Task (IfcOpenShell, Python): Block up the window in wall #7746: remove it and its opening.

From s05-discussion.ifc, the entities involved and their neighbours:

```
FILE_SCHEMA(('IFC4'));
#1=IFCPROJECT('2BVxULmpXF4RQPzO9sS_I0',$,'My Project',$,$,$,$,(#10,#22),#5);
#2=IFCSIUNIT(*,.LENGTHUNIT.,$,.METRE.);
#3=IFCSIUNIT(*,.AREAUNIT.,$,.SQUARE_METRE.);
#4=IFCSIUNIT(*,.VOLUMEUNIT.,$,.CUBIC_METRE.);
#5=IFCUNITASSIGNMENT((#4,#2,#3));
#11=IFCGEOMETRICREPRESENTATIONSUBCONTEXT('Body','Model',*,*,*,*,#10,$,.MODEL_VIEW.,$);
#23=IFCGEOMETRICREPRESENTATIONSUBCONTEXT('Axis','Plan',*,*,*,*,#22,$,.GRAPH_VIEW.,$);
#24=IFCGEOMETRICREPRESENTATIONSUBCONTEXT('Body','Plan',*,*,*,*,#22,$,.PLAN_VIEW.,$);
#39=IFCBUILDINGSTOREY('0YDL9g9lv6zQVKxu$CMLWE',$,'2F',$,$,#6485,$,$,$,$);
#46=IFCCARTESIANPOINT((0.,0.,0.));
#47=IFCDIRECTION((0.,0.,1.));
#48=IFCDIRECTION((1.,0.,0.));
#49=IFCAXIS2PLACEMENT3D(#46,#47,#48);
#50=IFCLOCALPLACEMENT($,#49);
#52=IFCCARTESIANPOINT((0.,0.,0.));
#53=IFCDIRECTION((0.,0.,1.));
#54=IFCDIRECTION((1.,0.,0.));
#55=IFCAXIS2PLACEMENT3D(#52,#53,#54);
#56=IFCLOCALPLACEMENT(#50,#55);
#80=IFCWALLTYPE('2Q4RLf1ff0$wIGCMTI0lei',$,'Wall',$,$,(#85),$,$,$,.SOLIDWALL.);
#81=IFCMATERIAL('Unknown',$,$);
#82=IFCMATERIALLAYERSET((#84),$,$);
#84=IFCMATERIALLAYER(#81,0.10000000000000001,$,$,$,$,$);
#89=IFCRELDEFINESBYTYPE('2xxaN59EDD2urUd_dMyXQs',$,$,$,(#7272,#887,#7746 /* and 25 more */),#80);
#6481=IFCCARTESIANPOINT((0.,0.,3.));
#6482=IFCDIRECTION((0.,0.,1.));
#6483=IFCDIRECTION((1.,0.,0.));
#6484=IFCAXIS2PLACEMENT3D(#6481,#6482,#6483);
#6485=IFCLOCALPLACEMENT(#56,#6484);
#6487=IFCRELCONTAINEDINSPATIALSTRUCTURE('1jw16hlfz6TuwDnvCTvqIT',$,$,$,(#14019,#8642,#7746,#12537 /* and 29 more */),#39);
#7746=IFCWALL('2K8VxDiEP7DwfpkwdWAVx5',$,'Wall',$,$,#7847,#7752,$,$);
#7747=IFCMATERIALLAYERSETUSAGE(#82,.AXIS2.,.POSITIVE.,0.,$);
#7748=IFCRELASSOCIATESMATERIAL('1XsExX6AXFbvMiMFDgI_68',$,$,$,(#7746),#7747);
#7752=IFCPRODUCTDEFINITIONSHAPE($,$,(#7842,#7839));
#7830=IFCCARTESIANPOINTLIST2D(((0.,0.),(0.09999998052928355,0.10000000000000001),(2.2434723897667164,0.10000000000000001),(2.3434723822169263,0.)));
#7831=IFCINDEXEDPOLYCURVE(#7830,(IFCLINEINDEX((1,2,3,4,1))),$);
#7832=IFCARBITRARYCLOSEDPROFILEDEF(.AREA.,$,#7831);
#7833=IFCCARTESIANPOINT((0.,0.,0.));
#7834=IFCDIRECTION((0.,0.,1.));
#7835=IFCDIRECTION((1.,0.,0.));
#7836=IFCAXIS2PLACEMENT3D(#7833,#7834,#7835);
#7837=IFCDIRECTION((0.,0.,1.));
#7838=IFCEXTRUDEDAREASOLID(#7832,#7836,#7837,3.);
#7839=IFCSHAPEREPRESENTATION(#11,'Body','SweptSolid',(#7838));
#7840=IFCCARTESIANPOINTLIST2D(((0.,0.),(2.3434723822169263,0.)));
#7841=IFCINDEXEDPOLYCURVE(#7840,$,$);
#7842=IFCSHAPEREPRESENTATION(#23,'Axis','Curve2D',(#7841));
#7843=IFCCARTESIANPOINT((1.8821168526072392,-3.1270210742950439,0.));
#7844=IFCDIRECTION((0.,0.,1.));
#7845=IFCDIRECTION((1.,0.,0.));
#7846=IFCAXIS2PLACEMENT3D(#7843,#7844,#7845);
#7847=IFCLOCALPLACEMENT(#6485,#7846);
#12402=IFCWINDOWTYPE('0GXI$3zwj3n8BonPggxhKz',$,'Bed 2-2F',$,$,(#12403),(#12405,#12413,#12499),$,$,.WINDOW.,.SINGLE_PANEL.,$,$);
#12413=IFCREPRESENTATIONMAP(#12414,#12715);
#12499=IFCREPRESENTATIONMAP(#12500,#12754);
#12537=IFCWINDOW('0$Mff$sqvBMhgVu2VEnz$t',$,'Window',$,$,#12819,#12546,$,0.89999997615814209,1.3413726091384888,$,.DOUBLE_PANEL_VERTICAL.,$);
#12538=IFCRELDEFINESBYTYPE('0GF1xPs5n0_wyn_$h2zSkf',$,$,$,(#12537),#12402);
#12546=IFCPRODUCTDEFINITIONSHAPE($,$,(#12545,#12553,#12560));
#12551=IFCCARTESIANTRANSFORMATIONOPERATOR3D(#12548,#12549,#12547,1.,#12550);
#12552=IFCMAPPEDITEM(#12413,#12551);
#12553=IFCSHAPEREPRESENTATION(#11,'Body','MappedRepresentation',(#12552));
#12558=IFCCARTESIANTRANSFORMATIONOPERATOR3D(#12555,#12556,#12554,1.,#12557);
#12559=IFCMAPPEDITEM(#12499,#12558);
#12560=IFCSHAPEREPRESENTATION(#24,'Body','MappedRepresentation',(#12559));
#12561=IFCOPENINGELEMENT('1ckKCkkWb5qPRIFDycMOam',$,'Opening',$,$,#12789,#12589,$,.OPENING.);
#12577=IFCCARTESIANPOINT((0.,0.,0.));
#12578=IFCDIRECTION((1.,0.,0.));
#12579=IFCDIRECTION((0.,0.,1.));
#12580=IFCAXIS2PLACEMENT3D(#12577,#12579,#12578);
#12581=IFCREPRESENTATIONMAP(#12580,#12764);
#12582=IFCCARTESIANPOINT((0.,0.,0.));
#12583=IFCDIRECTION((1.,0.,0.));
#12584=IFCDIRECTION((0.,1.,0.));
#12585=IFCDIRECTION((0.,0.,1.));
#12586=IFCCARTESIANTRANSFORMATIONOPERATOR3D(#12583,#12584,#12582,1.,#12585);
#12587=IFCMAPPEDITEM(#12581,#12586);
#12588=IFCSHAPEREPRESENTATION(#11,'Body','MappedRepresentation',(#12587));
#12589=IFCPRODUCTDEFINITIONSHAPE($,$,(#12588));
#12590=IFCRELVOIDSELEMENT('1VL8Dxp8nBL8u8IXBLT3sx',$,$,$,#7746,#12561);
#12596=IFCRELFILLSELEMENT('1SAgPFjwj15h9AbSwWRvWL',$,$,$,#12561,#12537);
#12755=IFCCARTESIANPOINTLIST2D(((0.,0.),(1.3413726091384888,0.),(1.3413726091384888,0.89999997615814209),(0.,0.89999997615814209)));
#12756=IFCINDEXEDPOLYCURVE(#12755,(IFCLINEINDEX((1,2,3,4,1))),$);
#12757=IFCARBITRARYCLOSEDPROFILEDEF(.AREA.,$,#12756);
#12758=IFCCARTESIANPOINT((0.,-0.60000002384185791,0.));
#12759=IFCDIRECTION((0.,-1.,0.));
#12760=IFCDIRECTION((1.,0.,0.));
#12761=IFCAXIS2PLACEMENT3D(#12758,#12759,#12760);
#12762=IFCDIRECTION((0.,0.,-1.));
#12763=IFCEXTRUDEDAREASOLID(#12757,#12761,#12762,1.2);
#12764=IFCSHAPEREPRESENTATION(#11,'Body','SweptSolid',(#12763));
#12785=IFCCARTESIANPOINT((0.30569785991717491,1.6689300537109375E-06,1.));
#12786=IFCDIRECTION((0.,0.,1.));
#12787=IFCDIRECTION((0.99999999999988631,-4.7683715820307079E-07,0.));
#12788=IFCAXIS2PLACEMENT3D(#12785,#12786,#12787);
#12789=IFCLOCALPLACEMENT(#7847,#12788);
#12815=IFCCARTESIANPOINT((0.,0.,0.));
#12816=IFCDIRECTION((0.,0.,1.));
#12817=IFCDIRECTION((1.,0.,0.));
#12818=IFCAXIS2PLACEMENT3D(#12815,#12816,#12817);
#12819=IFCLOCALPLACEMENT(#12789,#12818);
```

```python
import ifcopenshell
import ifcopenshell.api.feature
import ifcopenshell.api.root
import ifcopenshell.geom
import ifcopenshell.util.shape

model = ifcopenshell.open("s05-discussion.ifc")
settings = ifcopenshell.geom.settings()


def volume(element):
    """Net volume in cubic metres, openings subtracted."""
    shape = ifcopenshell.geom.create_shape(settings, element)
    return ifcopenshell.util.shape.get_volume(shape.geometry)


window = model.by_guid("0$Mff$sqvBMhgVu2VEnz$t")
opening = window.FillsVoids[0].RelatingOpeningElement
wall = opening.VoidsElements[0].RelatingBuildingElement
before = volume(wall)

ifcopenshell.api.root.remove_product(model, product=window)
ifcopenshell.api.feature.remove_feature(model, feature=opening)

after = volume(wall)

print(f"wall volume {before:.3f} -> {after:.3f} m3")

model.write("s05-discussion_edited.ifc")
```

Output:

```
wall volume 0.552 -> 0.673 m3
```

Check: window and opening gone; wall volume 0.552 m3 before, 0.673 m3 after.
